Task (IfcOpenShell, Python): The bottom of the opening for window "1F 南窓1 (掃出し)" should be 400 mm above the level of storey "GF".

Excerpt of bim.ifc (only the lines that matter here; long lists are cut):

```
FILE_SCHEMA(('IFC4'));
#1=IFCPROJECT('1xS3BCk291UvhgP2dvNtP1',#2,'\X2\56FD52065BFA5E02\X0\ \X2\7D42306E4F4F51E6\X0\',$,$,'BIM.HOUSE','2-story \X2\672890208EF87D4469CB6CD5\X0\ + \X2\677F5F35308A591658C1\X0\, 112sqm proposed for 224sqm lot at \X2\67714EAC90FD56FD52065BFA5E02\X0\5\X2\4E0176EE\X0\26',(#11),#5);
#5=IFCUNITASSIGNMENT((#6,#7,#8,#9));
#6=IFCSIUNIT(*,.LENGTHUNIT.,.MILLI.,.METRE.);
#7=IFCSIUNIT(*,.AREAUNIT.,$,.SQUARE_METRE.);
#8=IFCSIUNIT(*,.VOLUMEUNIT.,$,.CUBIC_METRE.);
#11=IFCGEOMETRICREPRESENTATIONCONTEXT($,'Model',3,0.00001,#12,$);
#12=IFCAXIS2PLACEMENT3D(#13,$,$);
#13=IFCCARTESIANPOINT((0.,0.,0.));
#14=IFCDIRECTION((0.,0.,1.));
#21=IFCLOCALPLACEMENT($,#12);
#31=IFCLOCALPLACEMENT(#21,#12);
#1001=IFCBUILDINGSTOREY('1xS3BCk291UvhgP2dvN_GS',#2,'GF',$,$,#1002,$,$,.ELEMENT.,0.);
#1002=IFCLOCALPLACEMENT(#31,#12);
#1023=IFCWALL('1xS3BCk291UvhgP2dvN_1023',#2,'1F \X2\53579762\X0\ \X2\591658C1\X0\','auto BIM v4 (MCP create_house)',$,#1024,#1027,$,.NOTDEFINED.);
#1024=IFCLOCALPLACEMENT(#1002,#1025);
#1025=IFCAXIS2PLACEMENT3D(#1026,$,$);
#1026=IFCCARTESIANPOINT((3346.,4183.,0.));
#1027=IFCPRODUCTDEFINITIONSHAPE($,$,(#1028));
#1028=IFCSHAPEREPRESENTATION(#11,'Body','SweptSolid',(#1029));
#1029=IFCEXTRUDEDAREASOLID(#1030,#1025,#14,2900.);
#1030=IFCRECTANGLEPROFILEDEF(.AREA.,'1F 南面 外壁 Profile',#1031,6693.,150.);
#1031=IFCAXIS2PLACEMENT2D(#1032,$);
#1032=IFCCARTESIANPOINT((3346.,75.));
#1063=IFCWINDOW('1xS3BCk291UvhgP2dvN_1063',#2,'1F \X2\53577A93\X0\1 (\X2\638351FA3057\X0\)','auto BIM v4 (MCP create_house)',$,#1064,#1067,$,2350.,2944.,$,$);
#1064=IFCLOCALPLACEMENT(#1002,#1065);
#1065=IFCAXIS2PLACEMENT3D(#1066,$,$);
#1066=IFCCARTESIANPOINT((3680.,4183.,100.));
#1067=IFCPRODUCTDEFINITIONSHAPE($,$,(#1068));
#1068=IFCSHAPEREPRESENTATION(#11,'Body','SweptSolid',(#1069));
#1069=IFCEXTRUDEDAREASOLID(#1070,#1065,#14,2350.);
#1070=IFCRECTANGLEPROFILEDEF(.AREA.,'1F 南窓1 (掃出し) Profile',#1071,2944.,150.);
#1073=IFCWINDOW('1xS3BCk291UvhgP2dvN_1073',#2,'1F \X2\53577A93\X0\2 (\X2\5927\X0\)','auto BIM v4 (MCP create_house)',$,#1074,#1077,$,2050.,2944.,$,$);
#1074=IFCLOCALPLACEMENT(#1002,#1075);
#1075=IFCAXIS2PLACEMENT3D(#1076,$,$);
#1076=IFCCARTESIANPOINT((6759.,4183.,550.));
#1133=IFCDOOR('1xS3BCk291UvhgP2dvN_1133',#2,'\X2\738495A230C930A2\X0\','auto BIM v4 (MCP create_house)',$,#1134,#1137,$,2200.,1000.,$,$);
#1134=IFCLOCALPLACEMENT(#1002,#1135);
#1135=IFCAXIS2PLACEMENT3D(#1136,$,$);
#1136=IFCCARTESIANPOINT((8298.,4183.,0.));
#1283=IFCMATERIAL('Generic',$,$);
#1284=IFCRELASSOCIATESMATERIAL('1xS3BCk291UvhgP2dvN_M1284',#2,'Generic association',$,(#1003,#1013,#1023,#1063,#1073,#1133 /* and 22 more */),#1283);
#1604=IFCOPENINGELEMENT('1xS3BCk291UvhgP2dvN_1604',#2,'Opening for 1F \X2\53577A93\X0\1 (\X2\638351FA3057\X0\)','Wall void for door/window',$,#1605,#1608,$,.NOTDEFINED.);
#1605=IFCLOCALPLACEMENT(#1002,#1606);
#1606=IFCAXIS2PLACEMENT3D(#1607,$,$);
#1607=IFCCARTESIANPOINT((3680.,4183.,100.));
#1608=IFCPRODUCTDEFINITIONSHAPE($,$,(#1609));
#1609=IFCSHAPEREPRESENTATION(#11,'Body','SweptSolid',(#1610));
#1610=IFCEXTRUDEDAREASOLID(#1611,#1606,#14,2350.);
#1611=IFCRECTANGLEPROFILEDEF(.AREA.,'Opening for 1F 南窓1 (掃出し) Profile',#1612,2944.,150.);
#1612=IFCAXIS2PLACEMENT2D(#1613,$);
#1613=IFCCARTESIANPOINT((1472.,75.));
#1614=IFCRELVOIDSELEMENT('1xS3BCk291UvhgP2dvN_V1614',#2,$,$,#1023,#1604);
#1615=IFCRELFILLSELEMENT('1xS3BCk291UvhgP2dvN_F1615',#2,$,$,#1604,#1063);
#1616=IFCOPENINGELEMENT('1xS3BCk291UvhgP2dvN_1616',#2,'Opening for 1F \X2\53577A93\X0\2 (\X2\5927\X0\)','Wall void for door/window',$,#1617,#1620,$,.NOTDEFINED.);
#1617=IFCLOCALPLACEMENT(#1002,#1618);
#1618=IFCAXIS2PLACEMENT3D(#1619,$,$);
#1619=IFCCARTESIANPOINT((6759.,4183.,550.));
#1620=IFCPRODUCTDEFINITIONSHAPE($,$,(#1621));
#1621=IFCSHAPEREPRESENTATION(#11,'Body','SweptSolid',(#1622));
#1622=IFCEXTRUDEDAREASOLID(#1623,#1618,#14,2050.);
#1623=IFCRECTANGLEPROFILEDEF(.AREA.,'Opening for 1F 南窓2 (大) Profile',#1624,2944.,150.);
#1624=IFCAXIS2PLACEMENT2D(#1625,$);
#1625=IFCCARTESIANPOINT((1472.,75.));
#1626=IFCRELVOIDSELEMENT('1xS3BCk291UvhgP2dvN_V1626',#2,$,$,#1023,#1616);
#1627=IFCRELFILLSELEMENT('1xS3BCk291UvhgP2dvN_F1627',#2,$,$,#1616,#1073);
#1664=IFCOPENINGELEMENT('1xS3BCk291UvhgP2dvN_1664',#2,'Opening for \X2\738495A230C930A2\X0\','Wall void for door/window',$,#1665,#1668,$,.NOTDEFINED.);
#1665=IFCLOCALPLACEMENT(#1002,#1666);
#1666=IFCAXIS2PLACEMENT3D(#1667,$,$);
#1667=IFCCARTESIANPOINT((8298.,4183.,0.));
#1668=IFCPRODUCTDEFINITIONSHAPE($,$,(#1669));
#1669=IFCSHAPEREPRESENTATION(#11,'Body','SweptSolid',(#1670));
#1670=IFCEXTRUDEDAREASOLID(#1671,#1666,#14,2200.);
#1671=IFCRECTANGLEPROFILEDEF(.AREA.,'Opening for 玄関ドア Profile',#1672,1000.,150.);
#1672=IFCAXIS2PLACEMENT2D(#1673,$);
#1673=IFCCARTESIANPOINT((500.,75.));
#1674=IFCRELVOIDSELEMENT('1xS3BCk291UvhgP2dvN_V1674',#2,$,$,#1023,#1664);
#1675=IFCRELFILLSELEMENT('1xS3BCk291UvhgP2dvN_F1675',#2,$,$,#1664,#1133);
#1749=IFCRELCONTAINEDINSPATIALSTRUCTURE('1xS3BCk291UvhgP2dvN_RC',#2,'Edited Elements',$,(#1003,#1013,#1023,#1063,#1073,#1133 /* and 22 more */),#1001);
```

```python
import numpy as np
import ifcopenshell
import ifcopenshell.api.geometry
import ifcopenshell.geom
import ifcopenshell.util.element
import ifcopenshell.util.placement
import ifcopenshell.util.shape
import ifcopenshell.util.unit

model = ifcopenshell.open("bim.ifc")
unit_scale = ifcopenshell.util.unit.calculate_unit_scale(model)

window = model.by_guid("1xS3BCk291UvhgP2dvN_1063")
opening = window.FillsVoids[0].RelatingOpeningElement
storey = ifcopenshell.util.element.get_container(window, ifc_class="IfcBuildingStorey")
level = ifcopenshell.util.placement.get_local_placement(storey.ObjectPlacement)[2, 3]

# The opening's origin need not be at the sill, so measure its lowest point.
shape = ifcopenshell.geom.create_shape(ifcopenshell.geom.settings(), opening)
bottom = ifcopenshell.util.shape.get_shape_bottom_elevation(shape, shape.geometry) / unit_scale
dz = level + 0.4 / unit_scale - bottom

shift = np.array([0.0, 0.0, dz])
# The window is not placed relative to its opening, so move both.
for product in (opening, window):
    matrix = ifcopenshell.util.placement.get_local_placement(product.ObjectPlacement)
    matrix[:3, 3] += shift
    ifcopenshell.api.geometry.edit_object_placement(model, product=product, matrix=matrix, is_si=False)

print(f"moved by {dz * unit_scale:+.3f} m")

model.write("bim_v2.ifc")
```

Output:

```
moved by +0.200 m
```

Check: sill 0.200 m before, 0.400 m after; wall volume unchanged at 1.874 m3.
